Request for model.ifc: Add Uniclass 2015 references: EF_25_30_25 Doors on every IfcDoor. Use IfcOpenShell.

First a look at what the model holds.

```python
import ifcopenshell

model = ifcopenshell.open("model.ifc")
print(model.schema)
print("classifications:", [c.Name for c in model.by_type("IfcClassification")])
for ifc_class in ("IfcDoor", "IfcRoof", "IfcStair", "IfcWall", "IfcWindow"):
    print(ifc_class, len(model.by_type(ifc_class)))
```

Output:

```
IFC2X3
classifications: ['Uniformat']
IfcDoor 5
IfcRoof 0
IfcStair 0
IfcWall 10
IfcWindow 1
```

```python
import ifcopenshell
import ifcopenshell.api.classification

model = ifcopenshell.open("model.ifc")

# IFC2X3 requires Source and Edition and has no link from the project to the system.
system = model.create_entity("IfcClassification", Source="NBS", Edition="2015", Name="Uniclass 2015")

codes = {
    "IfcDoor": ("EF_25_30_25", "Doors"),
}
for ifc_class, (code, name) in codes.items():
    products = model.by_type(ifc_class)
    ifcopenshell.api.classification.add_reference(
        model, products=products, classification=system, identification=code, name=name
    )
    print(code, len(products))

model.write("model_v2.ifc")
```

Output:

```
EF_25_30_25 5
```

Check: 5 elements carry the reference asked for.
